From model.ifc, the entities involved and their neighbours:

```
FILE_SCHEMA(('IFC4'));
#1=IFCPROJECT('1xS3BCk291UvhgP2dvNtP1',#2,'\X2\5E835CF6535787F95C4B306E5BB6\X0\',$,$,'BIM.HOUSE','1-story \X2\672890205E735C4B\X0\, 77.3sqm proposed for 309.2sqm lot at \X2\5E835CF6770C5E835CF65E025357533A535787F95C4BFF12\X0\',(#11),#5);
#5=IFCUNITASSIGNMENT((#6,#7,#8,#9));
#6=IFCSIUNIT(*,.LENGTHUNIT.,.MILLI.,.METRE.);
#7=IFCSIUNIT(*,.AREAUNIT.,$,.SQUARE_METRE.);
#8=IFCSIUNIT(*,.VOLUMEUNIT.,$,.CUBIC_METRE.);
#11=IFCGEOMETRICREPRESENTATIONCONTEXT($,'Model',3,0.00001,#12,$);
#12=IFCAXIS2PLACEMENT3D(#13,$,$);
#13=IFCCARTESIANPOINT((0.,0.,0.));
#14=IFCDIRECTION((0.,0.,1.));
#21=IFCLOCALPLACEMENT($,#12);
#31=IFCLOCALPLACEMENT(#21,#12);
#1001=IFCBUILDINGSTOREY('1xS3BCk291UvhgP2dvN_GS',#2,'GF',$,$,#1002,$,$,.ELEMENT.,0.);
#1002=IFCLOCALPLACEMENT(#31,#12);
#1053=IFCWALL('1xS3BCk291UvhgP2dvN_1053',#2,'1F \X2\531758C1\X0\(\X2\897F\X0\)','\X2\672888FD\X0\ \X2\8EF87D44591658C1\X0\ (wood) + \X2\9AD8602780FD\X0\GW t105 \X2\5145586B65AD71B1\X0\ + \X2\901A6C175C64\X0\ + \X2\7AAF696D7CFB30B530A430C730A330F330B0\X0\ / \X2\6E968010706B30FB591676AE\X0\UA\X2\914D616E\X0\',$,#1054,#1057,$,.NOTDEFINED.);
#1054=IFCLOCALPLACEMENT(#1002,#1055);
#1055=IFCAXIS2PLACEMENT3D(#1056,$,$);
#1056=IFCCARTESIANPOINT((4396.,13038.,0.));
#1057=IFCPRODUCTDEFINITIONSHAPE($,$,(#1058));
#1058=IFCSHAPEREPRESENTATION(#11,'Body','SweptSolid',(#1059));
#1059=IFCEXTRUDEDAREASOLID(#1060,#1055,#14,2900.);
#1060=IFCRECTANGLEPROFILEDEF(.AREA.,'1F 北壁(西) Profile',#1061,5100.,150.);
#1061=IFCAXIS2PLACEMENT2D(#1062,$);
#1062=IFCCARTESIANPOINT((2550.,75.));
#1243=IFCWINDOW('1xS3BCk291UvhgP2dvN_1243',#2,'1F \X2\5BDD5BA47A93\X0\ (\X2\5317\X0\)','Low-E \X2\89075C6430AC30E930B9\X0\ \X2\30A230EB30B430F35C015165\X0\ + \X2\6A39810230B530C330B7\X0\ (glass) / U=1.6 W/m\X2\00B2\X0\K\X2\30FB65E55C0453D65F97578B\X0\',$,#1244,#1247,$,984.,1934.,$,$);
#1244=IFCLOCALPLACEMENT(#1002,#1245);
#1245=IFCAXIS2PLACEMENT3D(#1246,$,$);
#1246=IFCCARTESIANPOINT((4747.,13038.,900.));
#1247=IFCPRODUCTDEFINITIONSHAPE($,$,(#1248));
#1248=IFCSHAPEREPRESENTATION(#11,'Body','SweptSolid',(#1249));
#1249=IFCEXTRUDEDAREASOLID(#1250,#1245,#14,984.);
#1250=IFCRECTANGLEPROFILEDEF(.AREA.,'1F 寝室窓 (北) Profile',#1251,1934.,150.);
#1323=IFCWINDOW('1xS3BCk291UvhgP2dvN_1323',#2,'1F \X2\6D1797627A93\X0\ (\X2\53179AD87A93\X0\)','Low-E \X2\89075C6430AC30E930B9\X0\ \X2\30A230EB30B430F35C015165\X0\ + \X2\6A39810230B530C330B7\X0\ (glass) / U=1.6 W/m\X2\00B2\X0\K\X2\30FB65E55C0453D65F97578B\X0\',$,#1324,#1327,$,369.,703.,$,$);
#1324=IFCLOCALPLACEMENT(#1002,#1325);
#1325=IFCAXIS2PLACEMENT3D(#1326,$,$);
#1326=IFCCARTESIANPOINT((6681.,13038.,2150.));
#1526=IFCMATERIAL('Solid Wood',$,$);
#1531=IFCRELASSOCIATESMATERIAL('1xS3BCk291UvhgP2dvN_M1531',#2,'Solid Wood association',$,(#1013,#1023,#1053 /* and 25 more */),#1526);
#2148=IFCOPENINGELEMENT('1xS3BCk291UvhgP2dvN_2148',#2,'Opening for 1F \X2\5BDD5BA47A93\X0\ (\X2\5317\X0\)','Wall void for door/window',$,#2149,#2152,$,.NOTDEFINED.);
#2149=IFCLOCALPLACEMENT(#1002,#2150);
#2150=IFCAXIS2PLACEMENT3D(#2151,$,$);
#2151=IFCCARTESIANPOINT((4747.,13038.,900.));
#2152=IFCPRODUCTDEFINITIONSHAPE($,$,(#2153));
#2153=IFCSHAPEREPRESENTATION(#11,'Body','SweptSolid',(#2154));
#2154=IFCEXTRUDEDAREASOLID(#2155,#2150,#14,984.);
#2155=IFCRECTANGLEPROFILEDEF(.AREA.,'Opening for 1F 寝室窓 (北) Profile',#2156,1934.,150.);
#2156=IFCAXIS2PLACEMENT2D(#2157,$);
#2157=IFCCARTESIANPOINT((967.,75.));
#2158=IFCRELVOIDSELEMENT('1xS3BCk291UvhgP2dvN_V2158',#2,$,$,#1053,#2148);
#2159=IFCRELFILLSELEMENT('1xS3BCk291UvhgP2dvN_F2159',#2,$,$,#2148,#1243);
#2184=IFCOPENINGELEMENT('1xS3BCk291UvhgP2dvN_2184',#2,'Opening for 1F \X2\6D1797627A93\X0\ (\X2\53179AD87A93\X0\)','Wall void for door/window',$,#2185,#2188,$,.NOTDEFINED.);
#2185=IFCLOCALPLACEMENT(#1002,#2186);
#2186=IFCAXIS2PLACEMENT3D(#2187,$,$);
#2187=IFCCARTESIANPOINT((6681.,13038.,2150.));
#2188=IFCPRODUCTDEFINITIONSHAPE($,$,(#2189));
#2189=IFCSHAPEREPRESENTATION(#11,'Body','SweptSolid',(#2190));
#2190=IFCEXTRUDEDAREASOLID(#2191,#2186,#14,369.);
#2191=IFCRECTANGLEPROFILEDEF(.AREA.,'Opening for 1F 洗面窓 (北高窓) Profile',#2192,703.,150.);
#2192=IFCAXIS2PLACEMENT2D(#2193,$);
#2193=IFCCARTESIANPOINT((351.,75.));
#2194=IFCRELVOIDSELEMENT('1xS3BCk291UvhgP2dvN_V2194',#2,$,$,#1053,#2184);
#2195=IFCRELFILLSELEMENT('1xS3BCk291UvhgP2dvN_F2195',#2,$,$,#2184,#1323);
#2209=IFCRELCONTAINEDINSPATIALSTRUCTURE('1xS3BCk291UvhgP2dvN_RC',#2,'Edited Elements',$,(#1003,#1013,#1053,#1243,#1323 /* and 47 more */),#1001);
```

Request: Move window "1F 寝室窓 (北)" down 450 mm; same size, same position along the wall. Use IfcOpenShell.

```python
import numpy as np
import ifcopenshell
import ifcopenshell.api.geometry
import ifcopenshell.util.placement
import ifcopenshell.util.unit

model = ifcopenshell.open("model.ifc")
unit_scale = ifcopenshell.util.unit.calculate_unit_scale(model)

window = model.by_id(1243)
opening = window.FillsVoids[0].RelatingOpeningElement
dz = -0.45 / unit_scale

shift = np.array([0.0, 0.0, dz])
# The window is not placed relative to its opening, so move both.
for product in (opening, window):
    matrix = ifcopenshell.util.placement.get_local_placement(product.ObjectPlacement)
    matrix[:3, 3] += shift
    ifcopenshell.api.geometry.edit_object_placement(model, product=product, matrix=matrix, is_si=False)

print(f"moved by {dz * unit_scale:+.3f} m")

model.write("model_edited.ifc")
```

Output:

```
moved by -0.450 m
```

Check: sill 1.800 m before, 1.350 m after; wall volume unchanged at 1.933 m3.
